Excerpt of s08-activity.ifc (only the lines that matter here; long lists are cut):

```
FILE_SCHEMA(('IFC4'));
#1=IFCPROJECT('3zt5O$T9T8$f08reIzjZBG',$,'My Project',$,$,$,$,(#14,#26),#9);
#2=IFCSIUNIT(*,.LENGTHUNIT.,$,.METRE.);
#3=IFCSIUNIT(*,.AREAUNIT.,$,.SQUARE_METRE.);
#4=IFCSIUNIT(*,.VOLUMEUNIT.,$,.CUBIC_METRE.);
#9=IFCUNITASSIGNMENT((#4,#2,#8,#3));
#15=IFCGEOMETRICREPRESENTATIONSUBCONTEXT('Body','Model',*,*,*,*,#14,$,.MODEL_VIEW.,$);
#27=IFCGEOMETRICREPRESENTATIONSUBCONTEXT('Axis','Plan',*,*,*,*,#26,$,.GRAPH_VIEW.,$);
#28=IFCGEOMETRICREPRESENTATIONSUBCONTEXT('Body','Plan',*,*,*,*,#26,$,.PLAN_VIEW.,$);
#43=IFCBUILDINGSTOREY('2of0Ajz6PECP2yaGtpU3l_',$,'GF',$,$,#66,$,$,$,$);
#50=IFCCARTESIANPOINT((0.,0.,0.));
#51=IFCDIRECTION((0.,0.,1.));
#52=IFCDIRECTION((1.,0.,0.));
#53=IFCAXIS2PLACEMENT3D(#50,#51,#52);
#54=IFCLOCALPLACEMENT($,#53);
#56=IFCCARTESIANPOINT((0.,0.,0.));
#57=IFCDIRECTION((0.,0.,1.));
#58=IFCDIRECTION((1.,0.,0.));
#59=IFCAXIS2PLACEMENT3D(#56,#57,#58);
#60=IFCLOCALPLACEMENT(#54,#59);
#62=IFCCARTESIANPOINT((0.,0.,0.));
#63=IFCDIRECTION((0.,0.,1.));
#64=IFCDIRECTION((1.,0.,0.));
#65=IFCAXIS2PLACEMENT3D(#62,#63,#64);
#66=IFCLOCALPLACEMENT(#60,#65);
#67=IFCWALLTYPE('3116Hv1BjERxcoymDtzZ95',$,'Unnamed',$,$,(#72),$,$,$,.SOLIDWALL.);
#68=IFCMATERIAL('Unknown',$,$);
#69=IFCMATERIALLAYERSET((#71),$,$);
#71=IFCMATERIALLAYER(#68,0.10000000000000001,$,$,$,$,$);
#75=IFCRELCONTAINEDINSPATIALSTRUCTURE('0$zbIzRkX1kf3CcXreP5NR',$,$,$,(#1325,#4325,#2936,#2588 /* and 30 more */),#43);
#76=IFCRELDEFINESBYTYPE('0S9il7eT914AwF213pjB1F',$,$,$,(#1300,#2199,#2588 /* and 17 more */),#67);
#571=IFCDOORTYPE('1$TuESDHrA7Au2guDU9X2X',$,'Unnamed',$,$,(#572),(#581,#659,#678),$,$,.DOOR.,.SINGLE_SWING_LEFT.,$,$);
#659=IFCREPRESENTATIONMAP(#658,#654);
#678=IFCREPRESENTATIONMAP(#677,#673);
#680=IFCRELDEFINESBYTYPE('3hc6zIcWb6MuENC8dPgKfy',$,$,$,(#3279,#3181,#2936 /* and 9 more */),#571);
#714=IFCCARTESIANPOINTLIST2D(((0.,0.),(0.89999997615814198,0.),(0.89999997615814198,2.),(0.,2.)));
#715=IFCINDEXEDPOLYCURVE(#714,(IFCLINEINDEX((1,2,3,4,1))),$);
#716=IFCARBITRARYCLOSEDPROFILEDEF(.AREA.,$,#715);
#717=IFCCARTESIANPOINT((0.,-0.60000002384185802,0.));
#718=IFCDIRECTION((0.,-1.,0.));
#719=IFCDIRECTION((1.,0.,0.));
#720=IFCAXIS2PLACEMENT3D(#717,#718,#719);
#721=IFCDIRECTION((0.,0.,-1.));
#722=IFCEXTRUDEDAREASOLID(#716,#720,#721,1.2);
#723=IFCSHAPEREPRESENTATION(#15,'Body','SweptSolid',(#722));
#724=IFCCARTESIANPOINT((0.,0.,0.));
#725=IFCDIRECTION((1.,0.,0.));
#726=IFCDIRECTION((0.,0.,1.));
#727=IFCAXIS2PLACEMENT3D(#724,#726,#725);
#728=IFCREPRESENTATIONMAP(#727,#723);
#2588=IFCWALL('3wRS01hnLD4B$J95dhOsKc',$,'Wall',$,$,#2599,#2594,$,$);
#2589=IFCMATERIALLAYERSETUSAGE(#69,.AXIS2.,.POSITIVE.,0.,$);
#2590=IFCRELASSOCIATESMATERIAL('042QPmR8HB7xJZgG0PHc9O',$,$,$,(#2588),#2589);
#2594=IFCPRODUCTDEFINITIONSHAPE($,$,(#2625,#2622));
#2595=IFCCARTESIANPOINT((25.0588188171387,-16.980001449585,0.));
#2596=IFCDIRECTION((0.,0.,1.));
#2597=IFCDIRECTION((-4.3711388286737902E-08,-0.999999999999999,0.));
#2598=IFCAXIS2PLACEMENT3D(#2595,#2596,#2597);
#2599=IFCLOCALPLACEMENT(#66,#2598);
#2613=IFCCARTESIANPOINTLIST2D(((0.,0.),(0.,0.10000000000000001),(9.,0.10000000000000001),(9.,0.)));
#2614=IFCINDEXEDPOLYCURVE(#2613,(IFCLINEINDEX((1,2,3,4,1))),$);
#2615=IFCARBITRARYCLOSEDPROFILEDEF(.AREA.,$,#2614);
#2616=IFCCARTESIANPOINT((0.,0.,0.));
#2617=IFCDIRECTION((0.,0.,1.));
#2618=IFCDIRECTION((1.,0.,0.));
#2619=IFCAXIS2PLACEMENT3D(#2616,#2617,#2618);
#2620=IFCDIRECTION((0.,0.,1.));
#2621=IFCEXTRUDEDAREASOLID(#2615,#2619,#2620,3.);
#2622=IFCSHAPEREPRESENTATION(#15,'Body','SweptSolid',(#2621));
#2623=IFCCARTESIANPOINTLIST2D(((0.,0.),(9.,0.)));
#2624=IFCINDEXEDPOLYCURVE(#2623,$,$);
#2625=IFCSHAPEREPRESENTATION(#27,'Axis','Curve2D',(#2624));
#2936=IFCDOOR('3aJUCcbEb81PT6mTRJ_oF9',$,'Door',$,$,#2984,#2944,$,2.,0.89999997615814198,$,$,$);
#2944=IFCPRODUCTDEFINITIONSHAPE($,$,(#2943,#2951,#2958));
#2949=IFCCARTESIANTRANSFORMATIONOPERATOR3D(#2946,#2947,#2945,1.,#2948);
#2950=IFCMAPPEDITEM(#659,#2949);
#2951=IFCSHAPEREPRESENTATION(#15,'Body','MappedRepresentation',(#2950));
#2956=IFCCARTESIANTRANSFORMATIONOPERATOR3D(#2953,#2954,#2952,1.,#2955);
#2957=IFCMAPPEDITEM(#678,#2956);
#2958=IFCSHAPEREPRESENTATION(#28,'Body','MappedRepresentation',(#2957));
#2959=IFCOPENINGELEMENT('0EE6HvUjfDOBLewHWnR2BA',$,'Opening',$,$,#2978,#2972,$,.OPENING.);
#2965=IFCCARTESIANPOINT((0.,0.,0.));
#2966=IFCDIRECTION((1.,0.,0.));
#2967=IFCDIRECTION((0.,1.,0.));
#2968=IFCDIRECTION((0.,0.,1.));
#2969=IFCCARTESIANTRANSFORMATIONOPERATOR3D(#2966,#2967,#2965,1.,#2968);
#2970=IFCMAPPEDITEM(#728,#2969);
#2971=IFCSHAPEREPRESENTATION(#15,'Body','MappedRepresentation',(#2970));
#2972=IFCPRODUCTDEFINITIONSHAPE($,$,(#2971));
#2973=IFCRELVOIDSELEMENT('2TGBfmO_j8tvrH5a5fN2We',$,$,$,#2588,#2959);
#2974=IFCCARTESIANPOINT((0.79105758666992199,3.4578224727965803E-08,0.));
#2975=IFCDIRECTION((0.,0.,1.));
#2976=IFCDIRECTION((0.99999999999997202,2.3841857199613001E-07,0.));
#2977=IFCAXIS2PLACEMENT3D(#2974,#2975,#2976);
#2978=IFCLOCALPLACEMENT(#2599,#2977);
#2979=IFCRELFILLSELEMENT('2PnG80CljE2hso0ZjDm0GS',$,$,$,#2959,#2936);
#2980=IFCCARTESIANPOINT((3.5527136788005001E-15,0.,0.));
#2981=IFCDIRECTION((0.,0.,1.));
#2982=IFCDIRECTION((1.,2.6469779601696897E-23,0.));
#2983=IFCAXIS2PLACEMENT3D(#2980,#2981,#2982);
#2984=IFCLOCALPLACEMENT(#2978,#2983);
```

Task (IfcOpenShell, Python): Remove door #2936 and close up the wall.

```python
import ifcopenshell
import ifcopenshell.api.feature
import ifcopenshell.api.root
import ifcopenshell.geom
import ifcopenshell.util.shape

model = ifcopenshell.open("s08-activity.ifc")
settings = ifcopenshell.geom.settings()


def volume(element):
    """Net volume in cubic metres, openings subtracted."""
    shape = ifcopenshell.geom.create_shape(settings, element)
    return ifcopenshell.util.shape.get_volume(shape.geometry)


door = model.by_guid("3aJUCcbEb81PT6mTRJ_oF9")
opening = door.FillsVoids[0].RelatingOpeningElement
wall = opening.VoidsElements[0].RelatingBuildingElement
before = volume(wall)

ifcopenshell.api.root.remove_product(model, product=door)
ifcopenshell.api.feature.remove_feature(model, feature=opening)

after = volume(wall)

print(f"wall volume {before:.3f} -> {after:.3f} m3")

model.write("s08-activity_updated.ifc")
```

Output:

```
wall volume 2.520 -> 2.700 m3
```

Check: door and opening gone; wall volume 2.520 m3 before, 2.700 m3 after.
